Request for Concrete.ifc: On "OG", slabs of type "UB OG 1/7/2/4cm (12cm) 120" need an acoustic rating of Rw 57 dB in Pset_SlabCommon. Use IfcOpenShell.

First a look at what the model holds.

```python
import ifcopenshell
import ifcopenshell.util.element

model = ifcopenshell.open("Concrete.ifc")
print(model.schema)
storey = next(s for s in model.by_type("IfcBuildingStorey") if s.Name == "OG")
slabs = [e for e in ifcopenshell.util.element.get_decomposition(storey) if e.is_a("IfcSlab")]
seen = {}
for e in slabs:
    element_type = ifcopenshell.util.element.get_type(e)
    key = (element_type.Name if element_type != e and element_type else None, ifcopenshell.util.element.get_pset(e, "Pset_SlabCommon", "AcousticRating"))
    seen[key] = seen.get(key, 0) + 1
for (name, value), count in sorted(seen.items(), key=str):
    print(count, "x", name, "|", value)
```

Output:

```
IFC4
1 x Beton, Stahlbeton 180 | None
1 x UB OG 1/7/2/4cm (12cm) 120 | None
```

```python
import ifcopenshell
import ifcopenshell.api.pset
import ifcopenshell.util.element

model = ifcopenshell.open("Concrete.ifc")

storey = next(s for s in model.by_type("IfcBuildingStorey") if s.Name == "OG")
slabs = [e for e in ifcopenshell.util.element.get_decomposition(storey) if e.is_a("IfcSlab")]

count = 0
for e in slabs:
    element_type = ifcopenshell.util.element.get_type(e)
    if element_type in (None, e) or element_type.Name != "UB OG 1/7/2/4cm (12cm) 120":
        continue
    # add_pset returns the element's existing set when there is one.
    pset = ifcopenshell.api.pset.add_pset(model, product=e, name="Pset_SlabCommon")
    ifcopenshell.api.pset.edit_pset(model, pset=pset, properties={"AcousticRating": "Rw 57 dB"})
    count += 1

print(count, "slabs updated")

model.write("Concrete_rev.ifc")
```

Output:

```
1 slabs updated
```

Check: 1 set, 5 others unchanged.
